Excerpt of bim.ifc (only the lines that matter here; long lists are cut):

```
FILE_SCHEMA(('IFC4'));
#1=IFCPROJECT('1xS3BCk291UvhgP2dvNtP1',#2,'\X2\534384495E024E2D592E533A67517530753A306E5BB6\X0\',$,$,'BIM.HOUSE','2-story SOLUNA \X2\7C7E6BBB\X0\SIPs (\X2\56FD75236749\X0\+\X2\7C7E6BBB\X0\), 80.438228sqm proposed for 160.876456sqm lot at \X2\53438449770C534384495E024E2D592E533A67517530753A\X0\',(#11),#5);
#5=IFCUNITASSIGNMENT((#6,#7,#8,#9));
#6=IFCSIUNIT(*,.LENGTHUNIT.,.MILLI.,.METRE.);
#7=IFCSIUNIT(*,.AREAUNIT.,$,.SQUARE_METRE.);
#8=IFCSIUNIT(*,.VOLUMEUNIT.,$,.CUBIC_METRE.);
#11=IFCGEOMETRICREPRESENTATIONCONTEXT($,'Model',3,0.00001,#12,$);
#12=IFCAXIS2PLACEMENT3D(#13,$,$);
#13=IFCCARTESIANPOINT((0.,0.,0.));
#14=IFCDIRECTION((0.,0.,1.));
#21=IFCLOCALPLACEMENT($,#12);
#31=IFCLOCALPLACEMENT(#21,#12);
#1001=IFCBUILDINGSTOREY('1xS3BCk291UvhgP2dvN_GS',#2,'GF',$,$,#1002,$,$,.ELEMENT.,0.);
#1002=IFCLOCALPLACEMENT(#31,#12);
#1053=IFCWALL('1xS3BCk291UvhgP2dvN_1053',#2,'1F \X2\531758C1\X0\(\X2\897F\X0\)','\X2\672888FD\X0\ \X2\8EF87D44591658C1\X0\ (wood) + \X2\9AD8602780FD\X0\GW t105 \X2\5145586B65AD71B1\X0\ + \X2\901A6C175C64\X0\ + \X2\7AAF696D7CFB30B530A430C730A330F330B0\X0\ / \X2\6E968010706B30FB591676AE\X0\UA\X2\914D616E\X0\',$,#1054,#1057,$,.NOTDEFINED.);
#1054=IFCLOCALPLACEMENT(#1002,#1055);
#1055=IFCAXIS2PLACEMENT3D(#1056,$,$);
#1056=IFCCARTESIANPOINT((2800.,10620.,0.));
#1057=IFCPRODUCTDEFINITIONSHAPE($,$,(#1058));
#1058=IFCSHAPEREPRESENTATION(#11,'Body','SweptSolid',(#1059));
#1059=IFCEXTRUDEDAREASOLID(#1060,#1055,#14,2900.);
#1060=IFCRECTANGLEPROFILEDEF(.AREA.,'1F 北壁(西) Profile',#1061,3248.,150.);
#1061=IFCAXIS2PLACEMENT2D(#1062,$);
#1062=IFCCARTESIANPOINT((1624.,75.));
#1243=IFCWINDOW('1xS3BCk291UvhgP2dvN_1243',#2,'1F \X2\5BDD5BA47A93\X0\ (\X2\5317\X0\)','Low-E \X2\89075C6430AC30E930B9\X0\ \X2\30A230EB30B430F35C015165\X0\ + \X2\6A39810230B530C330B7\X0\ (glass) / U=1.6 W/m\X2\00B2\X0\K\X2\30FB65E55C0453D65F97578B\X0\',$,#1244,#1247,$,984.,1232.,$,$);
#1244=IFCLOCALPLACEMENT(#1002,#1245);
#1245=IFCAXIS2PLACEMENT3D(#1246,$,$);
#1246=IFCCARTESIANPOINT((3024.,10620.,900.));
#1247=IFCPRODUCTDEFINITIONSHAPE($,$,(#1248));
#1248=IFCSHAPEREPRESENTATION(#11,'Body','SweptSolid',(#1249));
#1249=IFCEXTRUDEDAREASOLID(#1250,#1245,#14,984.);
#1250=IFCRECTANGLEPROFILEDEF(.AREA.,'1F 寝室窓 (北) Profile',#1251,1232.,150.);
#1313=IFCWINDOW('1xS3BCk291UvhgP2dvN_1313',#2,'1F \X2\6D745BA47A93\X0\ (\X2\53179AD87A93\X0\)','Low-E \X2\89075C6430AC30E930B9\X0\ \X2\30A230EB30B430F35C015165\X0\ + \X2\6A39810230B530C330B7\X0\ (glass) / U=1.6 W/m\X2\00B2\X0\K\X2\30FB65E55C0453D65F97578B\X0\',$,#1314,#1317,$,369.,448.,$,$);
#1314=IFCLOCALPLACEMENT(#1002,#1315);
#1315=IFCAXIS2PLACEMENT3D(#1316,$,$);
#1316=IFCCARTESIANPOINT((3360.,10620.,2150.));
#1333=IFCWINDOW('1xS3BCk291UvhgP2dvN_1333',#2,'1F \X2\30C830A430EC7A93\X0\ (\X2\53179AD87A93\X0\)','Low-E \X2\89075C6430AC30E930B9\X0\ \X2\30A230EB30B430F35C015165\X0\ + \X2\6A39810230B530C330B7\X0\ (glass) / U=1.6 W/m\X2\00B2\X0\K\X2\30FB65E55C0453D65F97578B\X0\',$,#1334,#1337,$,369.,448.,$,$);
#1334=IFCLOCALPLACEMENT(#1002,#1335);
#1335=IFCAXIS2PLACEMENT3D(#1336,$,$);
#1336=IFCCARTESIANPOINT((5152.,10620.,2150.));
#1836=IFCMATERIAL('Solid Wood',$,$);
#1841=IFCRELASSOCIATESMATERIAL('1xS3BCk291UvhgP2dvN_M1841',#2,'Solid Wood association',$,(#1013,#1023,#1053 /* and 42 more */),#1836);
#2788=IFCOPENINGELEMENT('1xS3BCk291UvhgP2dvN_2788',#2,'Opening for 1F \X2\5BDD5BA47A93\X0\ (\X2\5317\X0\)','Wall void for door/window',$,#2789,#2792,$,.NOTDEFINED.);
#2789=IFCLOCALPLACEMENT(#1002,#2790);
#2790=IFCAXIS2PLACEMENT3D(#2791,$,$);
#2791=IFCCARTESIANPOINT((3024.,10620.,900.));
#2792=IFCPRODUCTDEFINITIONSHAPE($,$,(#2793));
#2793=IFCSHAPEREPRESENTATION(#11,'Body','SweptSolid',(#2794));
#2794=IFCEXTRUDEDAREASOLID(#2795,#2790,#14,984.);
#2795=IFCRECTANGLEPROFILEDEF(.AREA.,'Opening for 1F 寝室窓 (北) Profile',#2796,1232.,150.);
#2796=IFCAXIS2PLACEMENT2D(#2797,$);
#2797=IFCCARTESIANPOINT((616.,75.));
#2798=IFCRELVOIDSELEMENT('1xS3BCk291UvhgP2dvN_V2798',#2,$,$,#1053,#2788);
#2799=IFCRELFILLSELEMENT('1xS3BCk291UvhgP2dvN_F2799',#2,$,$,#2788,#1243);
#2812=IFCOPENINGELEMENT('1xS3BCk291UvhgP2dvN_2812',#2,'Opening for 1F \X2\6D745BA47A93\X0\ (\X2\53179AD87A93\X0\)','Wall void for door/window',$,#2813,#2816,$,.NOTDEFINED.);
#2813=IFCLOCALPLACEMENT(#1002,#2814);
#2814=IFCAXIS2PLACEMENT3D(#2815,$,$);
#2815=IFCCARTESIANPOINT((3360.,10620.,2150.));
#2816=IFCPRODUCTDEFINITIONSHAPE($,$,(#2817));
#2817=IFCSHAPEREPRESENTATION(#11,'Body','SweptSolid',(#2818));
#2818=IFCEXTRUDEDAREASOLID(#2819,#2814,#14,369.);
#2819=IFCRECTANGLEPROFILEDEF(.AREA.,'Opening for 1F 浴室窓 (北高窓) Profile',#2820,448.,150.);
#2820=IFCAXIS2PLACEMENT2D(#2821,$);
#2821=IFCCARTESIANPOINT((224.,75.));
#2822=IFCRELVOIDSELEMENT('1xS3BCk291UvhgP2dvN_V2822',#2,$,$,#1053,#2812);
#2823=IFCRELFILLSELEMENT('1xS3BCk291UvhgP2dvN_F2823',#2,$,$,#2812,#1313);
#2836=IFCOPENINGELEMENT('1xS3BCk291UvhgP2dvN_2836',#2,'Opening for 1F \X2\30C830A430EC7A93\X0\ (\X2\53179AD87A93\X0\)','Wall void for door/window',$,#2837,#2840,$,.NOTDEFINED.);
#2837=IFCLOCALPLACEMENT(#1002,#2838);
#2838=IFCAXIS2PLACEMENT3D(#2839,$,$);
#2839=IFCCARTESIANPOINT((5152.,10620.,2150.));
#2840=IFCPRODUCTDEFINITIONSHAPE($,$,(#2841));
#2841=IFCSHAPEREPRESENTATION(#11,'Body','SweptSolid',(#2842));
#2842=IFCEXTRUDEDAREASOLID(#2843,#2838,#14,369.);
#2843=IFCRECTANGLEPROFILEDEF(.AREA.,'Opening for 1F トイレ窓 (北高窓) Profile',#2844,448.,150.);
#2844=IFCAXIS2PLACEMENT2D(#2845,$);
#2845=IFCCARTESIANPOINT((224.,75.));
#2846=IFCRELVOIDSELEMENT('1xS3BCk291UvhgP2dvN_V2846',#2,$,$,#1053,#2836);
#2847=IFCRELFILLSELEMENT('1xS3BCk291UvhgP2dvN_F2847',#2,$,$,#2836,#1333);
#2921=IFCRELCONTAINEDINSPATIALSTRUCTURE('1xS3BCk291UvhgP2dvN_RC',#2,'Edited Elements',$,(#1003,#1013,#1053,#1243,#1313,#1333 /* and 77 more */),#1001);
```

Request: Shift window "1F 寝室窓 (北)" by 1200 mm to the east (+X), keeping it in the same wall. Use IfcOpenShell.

```python
import ifcopenshell
import ifcopenshell.api.geometry
import ifcopenshell.util.placement
import ifcopenshell.util.unit

model = ifcopenshell.open("bim.ifc")
unit_scale = ifcopenshell.util.unit.calculate_unit_scale(model)

window = model.by_id(1243)
opening = window.FillsVoids[0].RelatingOpeningElement
wall = opening.VoidsElements[0].RelatingBuildingElement

wall_matrix = ifcopenshell.util.placement.get_local_placement(wall.ObjectPlacement)
shift = wall_matrix[:3, 0] * 1.2 / unit_scale
before = ifcopenshell.util.placement.get_local_placement(window.ObjectPlacement)[:3, 3].copy()

# The window is not placed relative to its opening, so move both.
for product in (opening, window):
    matrix = ifcopenshell.util.placement.get_local_placement(product.ObjectPlacement)
    matrix[:3, 3] += shift
    ifcopenshell.api.geometry.edit_object_placement(model, product=product, matrix=matrix, is_si=False)

after = ifcopenshell.util.placement.get_local_placement(window.ObjectPlacement)[:3, 3]
print("window moved by", (after - before).round(3) + 0.0)

model.write("bim_v2.ifc")
```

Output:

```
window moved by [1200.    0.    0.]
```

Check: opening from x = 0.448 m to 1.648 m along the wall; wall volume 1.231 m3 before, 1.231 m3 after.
